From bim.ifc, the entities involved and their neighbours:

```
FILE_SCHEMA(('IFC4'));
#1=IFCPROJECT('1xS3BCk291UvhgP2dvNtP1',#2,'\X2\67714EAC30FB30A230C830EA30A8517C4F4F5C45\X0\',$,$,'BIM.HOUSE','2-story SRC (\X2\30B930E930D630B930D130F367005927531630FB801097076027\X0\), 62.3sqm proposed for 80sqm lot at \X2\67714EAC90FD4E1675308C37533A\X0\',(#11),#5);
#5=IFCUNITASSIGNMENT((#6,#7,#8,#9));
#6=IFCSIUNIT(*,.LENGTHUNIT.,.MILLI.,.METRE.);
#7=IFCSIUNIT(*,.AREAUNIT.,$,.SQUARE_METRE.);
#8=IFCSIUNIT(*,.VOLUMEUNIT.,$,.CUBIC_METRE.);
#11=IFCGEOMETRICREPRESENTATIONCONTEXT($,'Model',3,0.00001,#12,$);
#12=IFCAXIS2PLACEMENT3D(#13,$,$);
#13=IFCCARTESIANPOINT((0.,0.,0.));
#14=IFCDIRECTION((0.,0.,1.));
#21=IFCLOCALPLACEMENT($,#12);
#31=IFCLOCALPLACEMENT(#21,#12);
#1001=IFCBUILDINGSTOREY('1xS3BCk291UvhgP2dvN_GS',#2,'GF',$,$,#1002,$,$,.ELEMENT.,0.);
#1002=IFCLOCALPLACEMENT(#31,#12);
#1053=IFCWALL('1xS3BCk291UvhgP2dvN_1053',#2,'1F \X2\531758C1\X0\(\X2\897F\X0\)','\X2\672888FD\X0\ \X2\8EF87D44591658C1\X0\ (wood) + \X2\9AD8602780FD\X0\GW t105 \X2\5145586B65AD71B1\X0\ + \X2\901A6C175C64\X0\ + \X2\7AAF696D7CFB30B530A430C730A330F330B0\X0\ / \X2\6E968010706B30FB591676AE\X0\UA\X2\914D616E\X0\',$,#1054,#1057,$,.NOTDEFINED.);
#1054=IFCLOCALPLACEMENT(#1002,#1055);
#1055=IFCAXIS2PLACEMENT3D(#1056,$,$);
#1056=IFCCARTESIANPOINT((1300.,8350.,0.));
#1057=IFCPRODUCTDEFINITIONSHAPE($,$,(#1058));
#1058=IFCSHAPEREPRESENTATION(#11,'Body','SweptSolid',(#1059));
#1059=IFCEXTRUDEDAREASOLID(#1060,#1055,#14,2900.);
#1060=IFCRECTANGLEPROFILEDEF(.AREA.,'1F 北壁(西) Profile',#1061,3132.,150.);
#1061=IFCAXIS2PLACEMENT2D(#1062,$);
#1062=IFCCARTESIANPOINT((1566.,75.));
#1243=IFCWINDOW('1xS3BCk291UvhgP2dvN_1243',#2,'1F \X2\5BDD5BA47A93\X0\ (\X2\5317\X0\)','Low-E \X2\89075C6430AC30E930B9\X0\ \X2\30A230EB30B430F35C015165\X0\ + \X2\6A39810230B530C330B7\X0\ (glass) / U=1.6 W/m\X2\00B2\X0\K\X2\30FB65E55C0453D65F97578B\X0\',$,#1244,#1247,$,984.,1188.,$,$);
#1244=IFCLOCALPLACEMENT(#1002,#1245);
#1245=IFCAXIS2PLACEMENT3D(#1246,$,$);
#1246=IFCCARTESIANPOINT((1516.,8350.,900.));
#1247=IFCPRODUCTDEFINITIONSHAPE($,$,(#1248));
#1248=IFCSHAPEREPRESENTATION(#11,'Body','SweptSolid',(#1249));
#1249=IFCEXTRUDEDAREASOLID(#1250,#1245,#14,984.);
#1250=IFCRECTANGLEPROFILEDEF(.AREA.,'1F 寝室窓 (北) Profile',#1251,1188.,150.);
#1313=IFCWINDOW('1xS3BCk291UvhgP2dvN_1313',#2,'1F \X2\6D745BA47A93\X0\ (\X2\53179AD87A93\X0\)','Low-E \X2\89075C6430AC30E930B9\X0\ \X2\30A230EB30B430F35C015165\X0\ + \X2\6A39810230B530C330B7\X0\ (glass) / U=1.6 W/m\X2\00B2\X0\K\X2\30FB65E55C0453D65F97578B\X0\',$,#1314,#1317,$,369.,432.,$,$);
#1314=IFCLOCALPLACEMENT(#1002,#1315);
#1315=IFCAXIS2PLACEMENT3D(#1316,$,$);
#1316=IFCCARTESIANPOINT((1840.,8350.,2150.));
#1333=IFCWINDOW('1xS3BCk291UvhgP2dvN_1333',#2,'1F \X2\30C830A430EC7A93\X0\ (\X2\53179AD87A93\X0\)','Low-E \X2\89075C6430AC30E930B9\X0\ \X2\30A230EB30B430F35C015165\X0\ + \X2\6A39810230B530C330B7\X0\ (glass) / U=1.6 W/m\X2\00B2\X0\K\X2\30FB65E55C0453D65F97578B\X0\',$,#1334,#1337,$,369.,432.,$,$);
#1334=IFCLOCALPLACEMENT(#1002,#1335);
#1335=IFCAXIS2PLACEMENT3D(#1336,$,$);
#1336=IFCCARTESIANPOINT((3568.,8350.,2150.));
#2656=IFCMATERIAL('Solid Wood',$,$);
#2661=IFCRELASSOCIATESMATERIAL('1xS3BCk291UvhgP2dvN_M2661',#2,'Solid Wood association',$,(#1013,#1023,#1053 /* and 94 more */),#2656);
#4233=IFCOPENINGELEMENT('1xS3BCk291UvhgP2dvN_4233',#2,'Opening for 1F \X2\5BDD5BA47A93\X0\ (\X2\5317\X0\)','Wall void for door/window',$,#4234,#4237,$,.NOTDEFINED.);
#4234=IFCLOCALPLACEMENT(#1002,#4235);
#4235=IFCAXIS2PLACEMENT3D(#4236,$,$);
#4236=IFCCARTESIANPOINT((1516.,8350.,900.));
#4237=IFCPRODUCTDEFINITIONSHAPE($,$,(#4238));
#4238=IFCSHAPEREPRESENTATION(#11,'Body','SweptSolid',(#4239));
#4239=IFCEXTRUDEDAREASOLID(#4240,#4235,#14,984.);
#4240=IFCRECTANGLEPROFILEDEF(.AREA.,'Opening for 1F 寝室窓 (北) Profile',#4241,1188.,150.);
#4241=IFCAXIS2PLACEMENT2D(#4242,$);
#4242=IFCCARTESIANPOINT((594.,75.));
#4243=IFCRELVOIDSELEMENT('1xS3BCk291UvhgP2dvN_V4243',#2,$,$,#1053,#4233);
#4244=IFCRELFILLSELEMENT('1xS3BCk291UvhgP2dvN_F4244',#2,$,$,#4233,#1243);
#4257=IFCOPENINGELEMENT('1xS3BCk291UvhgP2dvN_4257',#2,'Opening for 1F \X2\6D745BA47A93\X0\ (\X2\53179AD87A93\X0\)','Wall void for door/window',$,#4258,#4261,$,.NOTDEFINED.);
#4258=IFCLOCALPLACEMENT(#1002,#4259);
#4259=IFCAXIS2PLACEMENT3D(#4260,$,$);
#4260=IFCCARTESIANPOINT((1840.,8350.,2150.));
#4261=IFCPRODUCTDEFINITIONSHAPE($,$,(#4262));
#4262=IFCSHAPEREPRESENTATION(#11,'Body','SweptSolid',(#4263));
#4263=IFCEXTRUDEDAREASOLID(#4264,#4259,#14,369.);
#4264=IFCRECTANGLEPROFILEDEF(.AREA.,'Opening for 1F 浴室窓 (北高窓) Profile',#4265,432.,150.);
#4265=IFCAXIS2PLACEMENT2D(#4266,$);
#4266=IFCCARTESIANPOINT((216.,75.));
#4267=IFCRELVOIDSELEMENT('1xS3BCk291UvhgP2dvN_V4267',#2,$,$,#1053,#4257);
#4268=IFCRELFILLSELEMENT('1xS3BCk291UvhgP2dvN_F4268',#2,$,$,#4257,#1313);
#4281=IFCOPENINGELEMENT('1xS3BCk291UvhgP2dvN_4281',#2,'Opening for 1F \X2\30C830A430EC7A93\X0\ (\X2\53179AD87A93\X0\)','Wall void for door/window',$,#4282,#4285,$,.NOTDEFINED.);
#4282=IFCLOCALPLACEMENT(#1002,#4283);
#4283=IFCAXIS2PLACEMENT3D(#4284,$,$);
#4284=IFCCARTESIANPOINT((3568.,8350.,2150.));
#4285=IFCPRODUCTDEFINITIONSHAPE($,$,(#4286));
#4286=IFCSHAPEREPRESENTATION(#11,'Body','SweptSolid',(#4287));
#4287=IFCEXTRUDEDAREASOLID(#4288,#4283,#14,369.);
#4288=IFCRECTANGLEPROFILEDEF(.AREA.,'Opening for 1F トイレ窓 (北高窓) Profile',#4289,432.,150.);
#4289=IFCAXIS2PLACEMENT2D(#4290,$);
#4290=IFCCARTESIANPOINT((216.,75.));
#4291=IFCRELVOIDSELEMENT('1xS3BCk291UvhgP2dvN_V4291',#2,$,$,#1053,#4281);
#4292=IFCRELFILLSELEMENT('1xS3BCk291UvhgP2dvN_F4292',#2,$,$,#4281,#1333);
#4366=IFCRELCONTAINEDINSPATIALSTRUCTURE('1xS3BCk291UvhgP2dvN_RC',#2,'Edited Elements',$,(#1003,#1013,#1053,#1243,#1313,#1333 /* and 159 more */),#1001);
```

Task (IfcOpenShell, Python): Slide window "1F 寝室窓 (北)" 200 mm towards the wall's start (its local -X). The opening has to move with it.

```python
import ifcopenshell
import ifcopenshell.api.geometry
import ifcopenshell.util.placement

model = ifcopenshell.open("bim.ifc")

window = model.by_id(1243)
opening = window.FillsVoids[0].RelatingOpeningElement
wall = opening.VoidsElements[0].RelatingBuildingElement

wall_matrix = ifcopenshell.util.placement.get_local_placement(wall.ObjectPlacement)
shift = wall_matrix[:3, 0] * -200.0
before = ifcopenshell.util.placement.get_local_placement(window.ObjectPlacement)[:3, 3].copy()

# The window is not placed relative to its opening, so move both.
for product in (opening, window):
    matrix = ifcopenshell.util.placement.get_local_placement(product.ObjectPlacement)
    matrix[:3, 3] += shift
    ifcopenshell.api.geometry.edit_object_placement(model, product=product, matrix=matrix, is_si=False)

after = ifcopenshell.util.placement.get_local_placement(window.ObjectPlacement)[:3, 3]
print("window moved by", (after - before).round(3) + 0.0)

model.write("bim_rev.ifc")
```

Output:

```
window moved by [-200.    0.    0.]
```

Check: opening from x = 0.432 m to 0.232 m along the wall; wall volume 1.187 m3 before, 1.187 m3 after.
